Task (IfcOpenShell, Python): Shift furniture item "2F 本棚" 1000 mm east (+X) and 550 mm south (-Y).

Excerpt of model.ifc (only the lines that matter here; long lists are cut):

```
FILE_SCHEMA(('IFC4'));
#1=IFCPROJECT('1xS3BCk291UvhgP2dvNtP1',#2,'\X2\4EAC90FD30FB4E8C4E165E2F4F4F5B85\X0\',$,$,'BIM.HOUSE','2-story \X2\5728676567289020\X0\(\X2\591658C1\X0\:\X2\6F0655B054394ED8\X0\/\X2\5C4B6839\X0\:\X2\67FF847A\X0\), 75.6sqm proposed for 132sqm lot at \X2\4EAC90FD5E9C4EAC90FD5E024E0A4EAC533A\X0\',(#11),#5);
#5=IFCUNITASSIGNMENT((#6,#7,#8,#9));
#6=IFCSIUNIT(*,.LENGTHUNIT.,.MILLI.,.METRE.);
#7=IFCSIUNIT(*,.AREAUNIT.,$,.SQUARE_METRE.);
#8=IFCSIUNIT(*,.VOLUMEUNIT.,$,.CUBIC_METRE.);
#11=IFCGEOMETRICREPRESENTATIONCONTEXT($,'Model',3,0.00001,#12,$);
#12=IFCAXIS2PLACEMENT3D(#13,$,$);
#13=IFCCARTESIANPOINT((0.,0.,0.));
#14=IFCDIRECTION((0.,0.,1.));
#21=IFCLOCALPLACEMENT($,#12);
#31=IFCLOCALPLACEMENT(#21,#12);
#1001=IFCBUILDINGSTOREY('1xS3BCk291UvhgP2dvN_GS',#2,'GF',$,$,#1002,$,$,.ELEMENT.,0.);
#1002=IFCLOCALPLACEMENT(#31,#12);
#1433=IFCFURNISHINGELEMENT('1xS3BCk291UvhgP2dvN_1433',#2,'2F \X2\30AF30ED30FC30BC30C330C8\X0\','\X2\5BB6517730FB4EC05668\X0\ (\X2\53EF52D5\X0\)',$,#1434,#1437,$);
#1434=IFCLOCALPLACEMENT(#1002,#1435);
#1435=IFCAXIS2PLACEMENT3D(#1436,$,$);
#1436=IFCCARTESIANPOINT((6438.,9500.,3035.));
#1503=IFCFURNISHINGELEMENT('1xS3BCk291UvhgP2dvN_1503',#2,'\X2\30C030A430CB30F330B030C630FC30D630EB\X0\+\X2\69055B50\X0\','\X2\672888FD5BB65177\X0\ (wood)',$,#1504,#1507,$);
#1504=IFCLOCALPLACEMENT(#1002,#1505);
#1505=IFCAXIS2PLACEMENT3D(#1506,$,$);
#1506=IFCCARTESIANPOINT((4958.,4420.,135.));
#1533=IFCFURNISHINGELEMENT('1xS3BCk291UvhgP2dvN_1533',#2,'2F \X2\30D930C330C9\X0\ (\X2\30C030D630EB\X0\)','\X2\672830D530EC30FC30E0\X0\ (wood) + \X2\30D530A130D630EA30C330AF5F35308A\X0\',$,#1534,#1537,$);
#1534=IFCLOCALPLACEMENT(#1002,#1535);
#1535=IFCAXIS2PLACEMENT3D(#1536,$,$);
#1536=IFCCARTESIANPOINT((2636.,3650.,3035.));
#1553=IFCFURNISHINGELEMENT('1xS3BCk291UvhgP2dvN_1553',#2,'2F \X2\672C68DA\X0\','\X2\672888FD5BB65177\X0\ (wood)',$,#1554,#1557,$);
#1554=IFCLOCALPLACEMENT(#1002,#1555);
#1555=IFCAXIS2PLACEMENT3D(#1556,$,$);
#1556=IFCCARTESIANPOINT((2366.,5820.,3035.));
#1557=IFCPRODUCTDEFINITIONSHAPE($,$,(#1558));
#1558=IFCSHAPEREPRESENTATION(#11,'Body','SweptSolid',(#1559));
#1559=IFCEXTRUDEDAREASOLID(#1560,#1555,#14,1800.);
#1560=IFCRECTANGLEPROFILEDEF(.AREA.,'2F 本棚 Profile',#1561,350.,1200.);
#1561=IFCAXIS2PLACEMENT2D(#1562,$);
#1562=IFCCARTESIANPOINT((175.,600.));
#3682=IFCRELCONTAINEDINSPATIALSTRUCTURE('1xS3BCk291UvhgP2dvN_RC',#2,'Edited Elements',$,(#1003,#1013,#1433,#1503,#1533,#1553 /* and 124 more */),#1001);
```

```python
import ifcopenshell
import ifcopenshell.api.geometry
import ifcopenshell.util.placement

model = ifcopenshell.open("model.ifc")

item = model.by_guid("1xS3BCk291UvhgP2dvN_1553")
matrix = ifcopenshell.util.placement.get_local_placement(item.ObjectPlacement)
matrix[0, 3] += 1000.0
matrix[1, 3] -= 550.0
ifcopenshell.api.geometry.edit_object_placement(model, product=item, matrix=matrix, is_si=False)

print(ifcopenshell.util.placement.get_local_placement(item.ObjectPlacement).round(3) + 0.0)

model.write("model_edited.ifc")
```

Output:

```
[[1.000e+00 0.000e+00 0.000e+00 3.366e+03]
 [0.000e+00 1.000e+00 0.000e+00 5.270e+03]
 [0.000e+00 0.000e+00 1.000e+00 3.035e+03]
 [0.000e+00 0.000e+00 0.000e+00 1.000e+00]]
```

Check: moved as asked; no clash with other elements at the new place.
